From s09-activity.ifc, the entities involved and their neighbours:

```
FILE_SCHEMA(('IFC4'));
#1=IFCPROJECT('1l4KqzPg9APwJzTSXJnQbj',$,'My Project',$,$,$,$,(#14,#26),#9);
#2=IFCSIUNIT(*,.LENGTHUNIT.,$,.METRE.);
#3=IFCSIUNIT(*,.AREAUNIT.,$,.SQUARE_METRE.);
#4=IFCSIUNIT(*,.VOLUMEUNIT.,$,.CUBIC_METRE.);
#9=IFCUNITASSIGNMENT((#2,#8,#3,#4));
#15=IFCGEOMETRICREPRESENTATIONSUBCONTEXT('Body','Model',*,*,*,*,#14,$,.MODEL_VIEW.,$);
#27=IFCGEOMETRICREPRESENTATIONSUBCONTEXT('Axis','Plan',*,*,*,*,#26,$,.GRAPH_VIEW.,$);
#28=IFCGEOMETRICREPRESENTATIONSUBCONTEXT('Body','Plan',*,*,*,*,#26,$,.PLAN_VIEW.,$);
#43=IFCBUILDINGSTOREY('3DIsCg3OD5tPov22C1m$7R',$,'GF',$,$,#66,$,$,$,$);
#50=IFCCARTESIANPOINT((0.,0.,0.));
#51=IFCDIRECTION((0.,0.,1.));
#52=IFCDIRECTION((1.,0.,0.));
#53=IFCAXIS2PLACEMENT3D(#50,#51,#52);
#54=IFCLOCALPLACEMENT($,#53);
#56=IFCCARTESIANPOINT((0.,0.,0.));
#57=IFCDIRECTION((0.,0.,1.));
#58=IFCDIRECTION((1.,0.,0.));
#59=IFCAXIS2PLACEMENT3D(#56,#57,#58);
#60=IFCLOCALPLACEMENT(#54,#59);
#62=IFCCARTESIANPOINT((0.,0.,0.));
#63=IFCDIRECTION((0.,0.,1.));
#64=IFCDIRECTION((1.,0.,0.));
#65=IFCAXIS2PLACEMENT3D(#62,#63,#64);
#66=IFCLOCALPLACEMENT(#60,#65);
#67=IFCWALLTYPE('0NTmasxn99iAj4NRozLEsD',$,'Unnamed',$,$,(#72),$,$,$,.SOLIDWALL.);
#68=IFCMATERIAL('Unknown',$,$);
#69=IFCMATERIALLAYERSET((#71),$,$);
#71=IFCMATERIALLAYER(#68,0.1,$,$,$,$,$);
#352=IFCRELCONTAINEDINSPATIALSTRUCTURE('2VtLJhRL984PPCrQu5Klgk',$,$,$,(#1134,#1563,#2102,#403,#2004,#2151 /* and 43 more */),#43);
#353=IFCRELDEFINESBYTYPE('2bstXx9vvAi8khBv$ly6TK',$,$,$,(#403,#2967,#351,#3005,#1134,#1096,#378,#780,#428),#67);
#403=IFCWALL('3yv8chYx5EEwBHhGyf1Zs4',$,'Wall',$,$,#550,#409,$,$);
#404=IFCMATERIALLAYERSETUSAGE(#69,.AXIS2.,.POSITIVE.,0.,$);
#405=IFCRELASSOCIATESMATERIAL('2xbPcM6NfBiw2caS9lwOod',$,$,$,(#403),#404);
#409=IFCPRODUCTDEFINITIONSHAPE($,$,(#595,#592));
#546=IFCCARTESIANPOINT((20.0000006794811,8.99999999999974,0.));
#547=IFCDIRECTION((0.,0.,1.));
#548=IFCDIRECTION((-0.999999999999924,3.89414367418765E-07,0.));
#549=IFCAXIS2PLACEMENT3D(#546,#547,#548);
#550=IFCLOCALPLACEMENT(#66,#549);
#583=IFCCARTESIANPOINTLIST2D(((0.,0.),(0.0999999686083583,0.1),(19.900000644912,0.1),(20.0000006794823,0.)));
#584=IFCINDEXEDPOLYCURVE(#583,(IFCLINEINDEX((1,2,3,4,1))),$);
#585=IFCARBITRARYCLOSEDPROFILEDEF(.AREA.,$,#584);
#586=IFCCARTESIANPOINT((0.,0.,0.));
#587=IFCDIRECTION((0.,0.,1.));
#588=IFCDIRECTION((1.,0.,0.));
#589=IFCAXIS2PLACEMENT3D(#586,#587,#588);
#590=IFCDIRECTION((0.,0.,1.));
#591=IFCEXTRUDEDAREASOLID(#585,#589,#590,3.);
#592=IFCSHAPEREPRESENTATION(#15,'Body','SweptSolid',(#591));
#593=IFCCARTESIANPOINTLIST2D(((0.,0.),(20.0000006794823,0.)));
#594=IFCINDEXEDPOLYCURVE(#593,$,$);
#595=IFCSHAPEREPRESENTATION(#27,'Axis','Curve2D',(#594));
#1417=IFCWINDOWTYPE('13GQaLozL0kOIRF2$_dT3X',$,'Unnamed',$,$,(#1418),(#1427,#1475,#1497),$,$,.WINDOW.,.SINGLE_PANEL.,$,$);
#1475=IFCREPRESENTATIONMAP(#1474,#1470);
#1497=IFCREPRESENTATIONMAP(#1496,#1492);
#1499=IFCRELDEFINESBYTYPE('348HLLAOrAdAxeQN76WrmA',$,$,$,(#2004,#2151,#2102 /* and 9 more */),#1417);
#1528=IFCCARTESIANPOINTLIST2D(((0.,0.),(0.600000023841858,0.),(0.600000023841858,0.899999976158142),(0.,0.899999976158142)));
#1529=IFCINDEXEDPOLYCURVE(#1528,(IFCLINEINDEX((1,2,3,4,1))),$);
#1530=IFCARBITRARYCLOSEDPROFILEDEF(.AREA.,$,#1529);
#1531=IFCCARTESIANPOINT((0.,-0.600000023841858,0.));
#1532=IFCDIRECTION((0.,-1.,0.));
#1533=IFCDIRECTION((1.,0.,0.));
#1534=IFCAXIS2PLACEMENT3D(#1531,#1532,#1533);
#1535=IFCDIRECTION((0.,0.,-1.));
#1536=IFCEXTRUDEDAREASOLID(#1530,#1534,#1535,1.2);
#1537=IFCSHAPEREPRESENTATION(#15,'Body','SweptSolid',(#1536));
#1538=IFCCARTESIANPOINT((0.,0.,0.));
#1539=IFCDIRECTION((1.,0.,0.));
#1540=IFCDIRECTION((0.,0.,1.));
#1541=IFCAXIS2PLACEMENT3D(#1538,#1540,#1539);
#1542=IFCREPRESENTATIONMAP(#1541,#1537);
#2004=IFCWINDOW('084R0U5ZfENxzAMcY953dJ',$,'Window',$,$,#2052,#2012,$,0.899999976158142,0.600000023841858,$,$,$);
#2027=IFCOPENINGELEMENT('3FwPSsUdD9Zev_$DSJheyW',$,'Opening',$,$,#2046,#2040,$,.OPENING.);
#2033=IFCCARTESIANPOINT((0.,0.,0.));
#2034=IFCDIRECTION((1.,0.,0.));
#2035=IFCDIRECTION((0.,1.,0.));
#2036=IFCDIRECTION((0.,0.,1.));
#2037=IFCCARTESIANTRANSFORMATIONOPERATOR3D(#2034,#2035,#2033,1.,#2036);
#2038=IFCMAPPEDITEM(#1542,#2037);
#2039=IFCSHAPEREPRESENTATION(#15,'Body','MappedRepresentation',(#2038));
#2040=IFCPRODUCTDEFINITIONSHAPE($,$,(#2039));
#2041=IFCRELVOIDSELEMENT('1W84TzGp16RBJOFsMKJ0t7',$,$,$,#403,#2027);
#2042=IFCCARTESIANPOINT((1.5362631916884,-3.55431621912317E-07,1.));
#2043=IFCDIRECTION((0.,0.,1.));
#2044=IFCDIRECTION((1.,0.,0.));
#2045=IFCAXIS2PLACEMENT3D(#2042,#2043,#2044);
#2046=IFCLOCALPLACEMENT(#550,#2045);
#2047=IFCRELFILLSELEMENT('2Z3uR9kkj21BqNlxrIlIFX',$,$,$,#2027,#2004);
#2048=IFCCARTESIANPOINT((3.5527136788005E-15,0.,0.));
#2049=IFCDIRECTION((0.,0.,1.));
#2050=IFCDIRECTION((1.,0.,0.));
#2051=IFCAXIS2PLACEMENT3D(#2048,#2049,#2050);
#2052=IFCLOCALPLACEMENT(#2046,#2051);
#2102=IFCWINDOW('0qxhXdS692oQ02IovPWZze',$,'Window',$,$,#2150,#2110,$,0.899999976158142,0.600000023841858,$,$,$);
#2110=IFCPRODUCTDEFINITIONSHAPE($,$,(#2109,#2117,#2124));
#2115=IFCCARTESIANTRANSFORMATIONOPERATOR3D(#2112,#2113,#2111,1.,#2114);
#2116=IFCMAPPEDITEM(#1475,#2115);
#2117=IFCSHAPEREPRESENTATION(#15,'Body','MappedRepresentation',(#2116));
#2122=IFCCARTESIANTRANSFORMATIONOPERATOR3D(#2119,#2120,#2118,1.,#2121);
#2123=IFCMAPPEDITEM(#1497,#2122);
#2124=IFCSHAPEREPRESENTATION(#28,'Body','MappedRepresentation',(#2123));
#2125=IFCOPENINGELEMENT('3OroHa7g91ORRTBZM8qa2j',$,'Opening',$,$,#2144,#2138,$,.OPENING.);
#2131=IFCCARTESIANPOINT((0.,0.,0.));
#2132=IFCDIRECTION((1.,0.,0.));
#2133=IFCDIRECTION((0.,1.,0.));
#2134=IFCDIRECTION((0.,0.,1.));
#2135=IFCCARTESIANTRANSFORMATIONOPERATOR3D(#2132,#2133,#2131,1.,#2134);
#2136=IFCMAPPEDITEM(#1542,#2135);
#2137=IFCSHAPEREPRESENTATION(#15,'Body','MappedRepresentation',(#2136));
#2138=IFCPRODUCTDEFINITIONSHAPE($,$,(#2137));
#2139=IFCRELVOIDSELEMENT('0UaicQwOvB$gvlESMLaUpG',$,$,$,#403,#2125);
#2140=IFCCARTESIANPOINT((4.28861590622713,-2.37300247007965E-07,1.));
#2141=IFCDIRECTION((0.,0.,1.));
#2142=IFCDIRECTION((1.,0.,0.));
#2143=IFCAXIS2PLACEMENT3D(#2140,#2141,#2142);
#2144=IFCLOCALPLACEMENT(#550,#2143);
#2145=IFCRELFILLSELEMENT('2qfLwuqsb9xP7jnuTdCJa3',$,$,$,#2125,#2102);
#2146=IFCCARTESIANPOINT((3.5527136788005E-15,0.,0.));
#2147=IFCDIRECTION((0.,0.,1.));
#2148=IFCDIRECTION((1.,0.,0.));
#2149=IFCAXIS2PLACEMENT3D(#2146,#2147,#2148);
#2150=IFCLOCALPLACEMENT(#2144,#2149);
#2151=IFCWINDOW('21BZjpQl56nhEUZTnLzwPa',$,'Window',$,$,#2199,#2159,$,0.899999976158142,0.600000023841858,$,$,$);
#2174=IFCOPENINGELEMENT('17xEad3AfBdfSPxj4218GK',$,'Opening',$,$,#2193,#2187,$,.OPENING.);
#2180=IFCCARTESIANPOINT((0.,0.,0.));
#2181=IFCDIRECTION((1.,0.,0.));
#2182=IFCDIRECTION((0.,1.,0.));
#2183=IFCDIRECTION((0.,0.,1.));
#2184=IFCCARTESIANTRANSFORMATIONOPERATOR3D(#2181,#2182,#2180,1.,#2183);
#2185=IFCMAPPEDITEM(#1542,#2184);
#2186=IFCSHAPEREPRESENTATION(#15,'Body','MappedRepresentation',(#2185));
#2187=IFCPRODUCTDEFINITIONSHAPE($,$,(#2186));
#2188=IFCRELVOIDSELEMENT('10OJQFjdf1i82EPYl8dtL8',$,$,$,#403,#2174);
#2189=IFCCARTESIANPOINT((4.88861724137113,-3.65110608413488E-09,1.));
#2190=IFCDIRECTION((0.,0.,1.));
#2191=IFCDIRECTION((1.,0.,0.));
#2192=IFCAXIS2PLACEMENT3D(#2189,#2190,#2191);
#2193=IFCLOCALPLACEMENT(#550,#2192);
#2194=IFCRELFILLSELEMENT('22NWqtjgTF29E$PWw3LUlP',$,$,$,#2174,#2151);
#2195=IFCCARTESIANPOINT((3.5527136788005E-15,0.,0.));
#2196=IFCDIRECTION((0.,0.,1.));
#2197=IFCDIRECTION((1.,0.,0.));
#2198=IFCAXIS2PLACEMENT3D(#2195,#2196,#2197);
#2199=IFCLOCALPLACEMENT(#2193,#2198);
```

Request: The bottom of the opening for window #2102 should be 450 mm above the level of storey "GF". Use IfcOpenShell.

```python
import numpy as np
import ifcopenshell
import ifcopenshell.api.geometry
import ifcopenshell.geom
import ifcopenshell.util.element
import ifcopenshell.util.placement
import ifcopenshell.util.shape
import ifcopenshell.util.unit

model = ifcopenshell.open("s09-activity.ifc")
unit_scale = ifcopenshell.util.unit.calculate_unit_scale(model)

window = model.by_guid("0qxhXdS692oQ02IovPWZze")
opening = window.FillsVoids[0].RelatingOpeningElement
storey = ifcopenshell.util.element.get_container(window, ifc_class="IfcBuildingStorey")
level = ifcopenshell.util.placement.get_local_placement(storey.ObjectPlacement)[2, 3]

# The opening's origin need not be at the sill, so measure its lowest point.
shape = ifcopenshell.geom.create_shape(ifcopenshell.geom.settings(), opening)
bottom = ifcopenshell.util.shape.get_shape_bottom_elevation(shape, shape.geometry) / unit_scale
dz = level + 0.45 / unit_scale - bottom

shift = np.array([0.0, 0.0, dz])
# The window is placed relative to its opening, so it follows when the opening moves.
matrix = ifcopenshell.util.placement.get_local_placement(opening.ObjectPlacement)
matrix[:3, 3] += shift
ifcopenshell.api.geometry.edit_object_placement(
    model, product=opening, matrix=matrix, is_si=False, should_transform_children=True
)

print(f"moved by {dz * unit_scale:+.3f} m")

model.write("s09-activity_updated.ifc")
```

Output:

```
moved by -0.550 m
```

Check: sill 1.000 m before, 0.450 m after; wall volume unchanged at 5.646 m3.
